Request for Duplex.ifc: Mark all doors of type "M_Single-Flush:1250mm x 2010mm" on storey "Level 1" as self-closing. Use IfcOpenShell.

First a look at what the model holds.

```python
import ifcopenshell
import ifcopenshell.util.element

model = ifcopenshell.open("Duplex.ifc")
print(model.schema)
storey = next(s for s in model.by_type("IfcBuildingStorey") if s.Name == "Level 1")
doors = [e for e in ifcopenshell.util.element.get_decomposition(storey) if e.is_a("IfcDoor")]
seen = {}
for e in doors:
    element_type = ifcopenshell.util.element.get_type(e)
    key = (element_type.Name if element_type != e and element_type else None, ifcopenshell.util.element.get_pset(e, "Pset_DoorCommon", "SelfClosing"))
    seen[key] = seen.get(key, 0) + 1
for (name, value), count in sorted(seen.items(), key=str):
    print(count, "x", name, "|", value)
```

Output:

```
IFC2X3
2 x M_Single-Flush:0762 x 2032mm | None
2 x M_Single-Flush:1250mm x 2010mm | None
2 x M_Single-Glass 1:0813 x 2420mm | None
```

```python
import ifcopenshell
import ifcopenshell.api.pset
import ifcopenshell.util.element

model = ifcopenshell.open("Duplex.ifc")

storey = next(s for s in model.by_type("IfcBuildingStorey") if s.Name == "Level 1")
doors = [e for e in ifcopenshell.util.element.get_decomposition(storey) if e.is_a("IfcDoor")]

count = 0
for e in doors:
    element_type = ifcopenshell.util.element.get_type(e)
    if element_type in (None, e) or element_type.Name != "M_Single-Flush:1250mm x 2010mm":
        continue
    # add_pset returns the element's existing set when there is one.
    pset = ifcopenshell.api.pset.add_pset(model, product=e, name="Pset_DoorCommon")
    ifcopenshell.api.pset.edit_pset(model, pset=pset, properties={"SelfClosing": True})
    count += 1

print(count, "doors updated")

model.write("Duplex_edited.ifc")
```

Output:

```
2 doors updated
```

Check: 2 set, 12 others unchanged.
